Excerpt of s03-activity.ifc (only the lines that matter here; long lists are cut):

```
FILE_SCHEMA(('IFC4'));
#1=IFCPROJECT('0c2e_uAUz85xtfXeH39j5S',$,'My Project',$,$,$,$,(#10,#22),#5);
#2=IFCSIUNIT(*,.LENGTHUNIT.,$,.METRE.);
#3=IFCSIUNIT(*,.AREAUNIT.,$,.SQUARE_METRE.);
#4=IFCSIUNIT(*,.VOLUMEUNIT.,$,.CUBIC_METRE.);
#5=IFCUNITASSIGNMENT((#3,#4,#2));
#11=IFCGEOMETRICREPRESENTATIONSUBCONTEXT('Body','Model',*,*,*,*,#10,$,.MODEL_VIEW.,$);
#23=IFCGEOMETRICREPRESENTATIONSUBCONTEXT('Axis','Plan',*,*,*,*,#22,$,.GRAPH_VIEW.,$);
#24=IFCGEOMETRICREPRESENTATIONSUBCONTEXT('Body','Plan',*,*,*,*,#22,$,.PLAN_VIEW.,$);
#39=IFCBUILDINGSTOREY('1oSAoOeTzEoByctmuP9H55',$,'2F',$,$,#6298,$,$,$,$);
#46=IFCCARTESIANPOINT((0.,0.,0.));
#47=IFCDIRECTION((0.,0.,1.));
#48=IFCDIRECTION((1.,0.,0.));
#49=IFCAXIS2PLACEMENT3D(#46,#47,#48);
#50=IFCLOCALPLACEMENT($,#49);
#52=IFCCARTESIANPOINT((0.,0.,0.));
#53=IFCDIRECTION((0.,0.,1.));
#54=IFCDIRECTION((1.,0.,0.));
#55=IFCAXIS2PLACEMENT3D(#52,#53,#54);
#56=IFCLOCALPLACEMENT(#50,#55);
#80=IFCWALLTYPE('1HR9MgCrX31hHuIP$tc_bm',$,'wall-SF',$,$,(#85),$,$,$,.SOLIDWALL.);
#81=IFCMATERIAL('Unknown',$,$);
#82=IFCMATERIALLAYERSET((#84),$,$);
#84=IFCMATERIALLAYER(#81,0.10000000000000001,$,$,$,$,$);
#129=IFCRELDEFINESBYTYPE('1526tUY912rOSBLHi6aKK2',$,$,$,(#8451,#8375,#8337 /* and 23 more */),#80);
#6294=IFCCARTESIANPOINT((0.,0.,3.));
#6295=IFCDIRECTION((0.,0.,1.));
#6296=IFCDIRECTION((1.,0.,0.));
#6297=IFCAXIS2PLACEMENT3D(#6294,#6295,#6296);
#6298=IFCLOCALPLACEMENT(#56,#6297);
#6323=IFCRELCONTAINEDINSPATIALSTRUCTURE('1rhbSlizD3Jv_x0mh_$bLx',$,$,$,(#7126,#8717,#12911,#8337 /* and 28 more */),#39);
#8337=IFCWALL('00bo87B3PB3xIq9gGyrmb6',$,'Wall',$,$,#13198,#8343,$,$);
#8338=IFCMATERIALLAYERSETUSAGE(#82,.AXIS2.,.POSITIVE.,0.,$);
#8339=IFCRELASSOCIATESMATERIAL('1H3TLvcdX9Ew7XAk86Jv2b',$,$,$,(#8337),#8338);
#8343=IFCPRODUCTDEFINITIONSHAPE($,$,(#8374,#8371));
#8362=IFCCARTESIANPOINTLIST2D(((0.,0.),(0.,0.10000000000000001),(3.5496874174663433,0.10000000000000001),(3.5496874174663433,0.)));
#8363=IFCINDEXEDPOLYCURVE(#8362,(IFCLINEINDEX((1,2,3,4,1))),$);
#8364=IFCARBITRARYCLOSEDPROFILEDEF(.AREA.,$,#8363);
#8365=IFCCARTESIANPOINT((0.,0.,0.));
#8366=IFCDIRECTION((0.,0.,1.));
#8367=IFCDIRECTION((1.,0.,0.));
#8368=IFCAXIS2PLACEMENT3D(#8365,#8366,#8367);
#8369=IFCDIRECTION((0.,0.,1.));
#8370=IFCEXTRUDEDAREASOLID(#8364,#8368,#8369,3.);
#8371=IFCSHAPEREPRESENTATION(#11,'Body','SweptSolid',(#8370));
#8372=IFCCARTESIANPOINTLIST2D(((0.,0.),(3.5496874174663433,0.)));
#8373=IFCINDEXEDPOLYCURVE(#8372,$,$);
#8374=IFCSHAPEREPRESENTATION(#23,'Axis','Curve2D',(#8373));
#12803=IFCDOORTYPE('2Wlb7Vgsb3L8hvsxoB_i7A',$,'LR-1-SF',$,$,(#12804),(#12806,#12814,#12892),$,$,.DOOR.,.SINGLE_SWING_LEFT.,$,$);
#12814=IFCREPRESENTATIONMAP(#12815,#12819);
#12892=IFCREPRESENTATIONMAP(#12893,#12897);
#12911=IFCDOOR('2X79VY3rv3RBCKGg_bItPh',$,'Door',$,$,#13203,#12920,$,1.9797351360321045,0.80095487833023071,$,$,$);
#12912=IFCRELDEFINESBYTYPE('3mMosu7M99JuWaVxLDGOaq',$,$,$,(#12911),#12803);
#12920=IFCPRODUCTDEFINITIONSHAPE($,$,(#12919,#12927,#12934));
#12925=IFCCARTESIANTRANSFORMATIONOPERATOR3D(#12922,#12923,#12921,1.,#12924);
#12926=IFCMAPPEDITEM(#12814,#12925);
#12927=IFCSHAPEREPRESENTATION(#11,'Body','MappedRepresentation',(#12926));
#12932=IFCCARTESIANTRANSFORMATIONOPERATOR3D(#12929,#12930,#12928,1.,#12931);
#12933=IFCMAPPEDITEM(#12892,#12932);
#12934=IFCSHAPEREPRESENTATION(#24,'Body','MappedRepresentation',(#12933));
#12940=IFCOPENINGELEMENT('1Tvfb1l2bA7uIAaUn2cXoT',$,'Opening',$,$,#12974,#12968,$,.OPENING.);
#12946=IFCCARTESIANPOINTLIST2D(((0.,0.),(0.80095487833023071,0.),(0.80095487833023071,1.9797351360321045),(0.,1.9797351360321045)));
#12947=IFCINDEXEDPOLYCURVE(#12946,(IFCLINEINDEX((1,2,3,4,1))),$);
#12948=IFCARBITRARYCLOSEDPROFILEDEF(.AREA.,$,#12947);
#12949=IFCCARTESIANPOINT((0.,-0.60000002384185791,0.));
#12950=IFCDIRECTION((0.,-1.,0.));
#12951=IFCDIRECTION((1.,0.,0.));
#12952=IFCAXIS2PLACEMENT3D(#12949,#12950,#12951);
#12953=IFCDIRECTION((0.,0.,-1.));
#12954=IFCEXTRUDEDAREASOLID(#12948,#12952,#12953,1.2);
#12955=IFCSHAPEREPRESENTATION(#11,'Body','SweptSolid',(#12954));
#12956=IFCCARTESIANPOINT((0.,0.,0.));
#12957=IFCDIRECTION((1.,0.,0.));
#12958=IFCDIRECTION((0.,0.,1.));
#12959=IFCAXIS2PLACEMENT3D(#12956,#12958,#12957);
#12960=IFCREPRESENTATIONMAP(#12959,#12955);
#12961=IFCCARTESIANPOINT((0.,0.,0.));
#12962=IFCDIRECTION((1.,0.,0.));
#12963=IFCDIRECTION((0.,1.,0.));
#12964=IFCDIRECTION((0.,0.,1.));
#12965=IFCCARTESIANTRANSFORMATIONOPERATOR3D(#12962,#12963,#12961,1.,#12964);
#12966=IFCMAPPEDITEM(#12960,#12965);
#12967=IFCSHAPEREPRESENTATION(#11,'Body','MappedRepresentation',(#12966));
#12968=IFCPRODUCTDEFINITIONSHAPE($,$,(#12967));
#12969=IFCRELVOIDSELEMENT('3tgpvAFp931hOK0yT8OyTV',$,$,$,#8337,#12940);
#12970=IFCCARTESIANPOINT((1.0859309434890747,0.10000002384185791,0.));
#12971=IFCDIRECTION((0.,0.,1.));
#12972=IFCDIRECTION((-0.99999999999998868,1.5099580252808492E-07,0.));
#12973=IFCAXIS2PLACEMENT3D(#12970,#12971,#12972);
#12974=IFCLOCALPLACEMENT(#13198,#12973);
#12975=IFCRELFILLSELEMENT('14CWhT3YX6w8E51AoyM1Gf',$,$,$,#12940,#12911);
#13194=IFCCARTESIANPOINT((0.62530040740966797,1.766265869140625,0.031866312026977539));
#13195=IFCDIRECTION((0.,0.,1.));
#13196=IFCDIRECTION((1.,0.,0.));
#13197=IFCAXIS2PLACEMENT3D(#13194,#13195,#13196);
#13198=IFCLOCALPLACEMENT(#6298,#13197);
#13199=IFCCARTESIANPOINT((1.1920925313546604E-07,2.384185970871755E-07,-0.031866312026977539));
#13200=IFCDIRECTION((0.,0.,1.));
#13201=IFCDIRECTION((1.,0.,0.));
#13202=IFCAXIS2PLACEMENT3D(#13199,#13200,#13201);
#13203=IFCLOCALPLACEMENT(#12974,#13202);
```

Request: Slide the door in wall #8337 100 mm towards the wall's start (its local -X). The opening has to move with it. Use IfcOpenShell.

```python
import ifcopenshell
import ifcopenshell.api.geometry
import ifcopenshell.util.placement
import ifcopenshell.util.unit

model = ifcopenshell.open("s03-activity.ifc")
unit_scale = ifcopenshell.util.unit.calculate_unit_scale(model)

door = model.by_guid("2X79VY3rv3RBCKGg_bItPh")
opening = door.FillsVoids[0].RelatingOpeningElement
wall = opening.VoidsElements[0].RelatingBuildingElement

wall_matrix = ifcopenshell.util.placement.get_local_placement(wall.ObjectPlacement)
shift = wall_matrix[:3, 0] * -0.1 / unit_scale
before = ifcopenshell.util.placement.get_local_placement(door.ObjectPlacement)[:3, 3].copy()

# The door is placed relative to its opening, so it follows when the opening moves.
matrix = ifcopenshell.util.placement.get_local_placement(opening.ObjectPlacement)
matrix[:3, 3] += shift
ifcopenshell.api.geometry.edit_object_placement(
    model, product=opening, matrix=matrix, is_si=False, should_transform_children=True
)

after = ifcopenshell.util.placement.get_local_placement(door.ObjectPlacement)[:3, 3]
print("door moved by", (after - before).round(3) + 0.0)

model.write("s03-activity_v2.ifc")
```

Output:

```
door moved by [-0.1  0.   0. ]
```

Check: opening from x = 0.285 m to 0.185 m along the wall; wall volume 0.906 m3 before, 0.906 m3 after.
